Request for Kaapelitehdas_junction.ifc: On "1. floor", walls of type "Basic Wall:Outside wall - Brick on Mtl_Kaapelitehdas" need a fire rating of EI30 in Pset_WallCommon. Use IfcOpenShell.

First a look at what the model holds.

```python
import ifcopenshell
import ifcopenshell.util.element

model = ifcopenshell.open("Kaapelitehdas_junction.ifc")
print(model.schema)
storey = next(s for s in model.by_type("IfcBuildingStorey") if s.Name == "1. floor")
walls = [e for e in ifcopenshell.util.element.get_decomposition(storey) if e.is_a("IfcWall")]
seen = {}
for e in walls:
    element_type = ifcopenshell.util.element.get_type(e)
    key = (element_type.Name if element_type != e and element_type else None, ifcopenshell.util.element.get_pset(e, "Pset_WallCommon", "FireRating"))
    seen[key] = seen.get(key, 0) + 1
for (name, value), count in sorted(seen.items(), key=str):
    print(count, "x", name, "|", value)
```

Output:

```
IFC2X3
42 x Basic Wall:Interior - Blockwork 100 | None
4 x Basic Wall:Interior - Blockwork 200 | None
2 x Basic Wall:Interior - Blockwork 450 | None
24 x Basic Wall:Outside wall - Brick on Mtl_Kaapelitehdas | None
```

```python
import ifcopenshell
import ifcopenshell.api.pset
import ifcopenshell.util.element

model = ifcopenshell.open("Kaapelitehdas_junction.ifc")

storey = next(s for s in model.by_type("IfcBuildingStorey") if s.Name == "1. floor")
walls = [e for e in ifcopenshell.util.element.get_decomposition(storey) if e.is_a("IfcWall")]

count = 0
for e in walls:
    element_type = ifcopenshell.util.element.get_type(e)
    if element_type in (None, e) or element_type.Name != "Basic Wall:Outside wall - Brick on Mtl_Kaapelitehdas":
        continue
    # add_pset returns the element's existing set when there is one.
    pset = ifcopenshell.api.pset.add_pset(model, product=e, name="Pset_WallCommon")
    ifcopenshell.api.pset.edit_pset(model, pset=pset, properties={"FireRating": "EI30"})
    count += 1

print(count, "walls updated")

model.write("Kaapelitehdas_junction_rev.ifc")
```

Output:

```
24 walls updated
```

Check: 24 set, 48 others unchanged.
